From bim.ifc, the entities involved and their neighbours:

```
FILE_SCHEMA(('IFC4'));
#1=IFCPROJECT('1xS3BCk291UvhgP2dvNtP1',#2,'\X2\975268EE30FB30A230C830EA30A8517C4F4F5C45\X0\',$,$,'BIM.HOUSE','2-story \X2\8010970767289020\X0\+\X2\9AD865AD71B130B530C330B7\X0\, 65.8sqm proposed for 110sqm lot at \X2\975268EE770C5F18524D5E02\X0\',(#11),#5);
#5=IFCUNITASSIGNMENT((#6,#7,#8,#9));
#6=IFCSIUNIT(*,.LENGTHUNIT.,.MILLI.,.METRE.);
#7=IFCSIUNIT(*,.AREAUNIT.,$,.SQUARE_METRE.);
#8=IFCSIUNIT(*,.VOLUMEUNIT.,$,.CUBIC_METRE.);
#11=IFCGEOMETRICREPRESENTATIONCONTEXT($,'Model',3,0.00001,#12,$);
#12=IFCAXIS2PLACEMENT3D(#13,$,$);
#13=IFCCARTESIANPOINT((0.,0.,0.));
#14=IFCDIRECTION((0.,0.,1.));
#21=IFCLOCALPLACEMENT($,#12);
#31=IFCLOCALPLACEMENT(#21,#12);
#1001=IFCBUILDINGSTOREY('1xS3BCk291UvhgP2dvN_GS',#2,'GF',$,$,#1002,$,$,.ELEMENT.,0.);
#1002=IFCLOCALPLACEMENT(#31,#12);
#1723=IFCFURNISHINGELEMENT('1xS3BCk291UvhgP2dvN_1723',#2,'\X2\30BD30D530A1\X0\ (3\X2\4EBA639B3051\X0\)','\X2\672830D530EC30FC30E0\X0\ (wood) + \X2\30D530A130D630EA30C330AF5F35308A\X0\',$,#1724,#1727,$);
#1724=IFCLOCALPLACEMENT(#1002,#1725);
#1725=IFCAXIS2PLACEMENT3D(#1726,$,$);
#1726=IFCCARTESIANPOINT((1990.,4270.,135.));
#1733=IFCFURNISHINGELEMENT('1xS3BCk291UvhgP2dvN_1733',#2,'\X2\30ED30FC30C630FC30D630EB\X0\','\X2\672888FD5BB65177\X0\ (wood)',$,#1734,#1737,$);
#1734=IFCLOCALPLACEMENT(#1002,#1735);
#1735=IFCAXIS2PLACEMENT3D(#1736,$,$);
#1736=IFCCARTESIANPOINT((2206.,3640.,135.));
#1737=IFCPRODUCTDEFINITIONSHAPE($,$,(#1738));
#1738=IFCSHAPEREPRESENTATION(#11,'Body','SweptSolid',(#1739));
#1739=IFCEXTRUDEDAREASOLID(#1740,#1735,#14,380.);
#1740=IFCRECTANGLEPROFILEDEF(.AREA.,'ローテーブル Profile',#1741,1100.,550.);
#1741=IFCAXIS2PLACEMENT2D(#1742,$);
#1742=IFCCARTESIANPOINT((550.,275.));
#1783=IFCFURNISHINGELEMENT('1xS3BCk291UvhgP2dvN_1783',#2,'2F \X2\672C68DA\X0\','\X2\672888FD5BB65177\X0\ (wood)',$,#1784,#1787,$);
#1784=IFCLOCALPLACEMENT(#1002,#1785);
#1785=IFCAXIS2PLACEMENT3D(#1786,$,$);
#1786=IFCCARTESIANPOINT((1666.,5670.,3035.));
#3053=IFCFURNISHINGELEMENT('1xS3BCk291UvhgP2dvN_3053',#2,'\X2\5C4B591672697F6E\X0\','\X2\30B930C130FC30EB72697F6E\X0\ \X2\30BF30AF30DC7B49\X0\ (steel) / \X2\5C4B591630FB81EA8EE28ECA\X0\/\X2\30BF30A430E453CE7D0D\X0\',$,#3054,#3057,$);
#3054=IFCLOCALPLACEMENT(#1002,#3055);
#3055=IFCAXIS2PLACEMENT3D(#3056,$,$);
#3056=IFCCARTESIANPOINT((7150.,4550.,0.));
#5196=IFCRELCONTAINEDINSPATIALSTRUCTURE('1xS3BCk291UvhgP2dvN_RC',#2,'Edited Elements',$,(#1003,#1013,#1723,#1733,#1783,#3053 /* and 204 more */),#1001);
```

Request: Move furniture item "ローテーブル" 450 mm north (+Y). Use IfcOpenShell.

```python
import ifcopenshell
import ifcopenshell.api.geometry
import ifcopenshell.util.placement
import ifcopenshell.util.unit

model = ifcopenshell.open("bim.ifc")
unit_scale = ifcopenshell.util.unit.calculate_unit_scale(model)

item = model.by_id(1733)
matrix = ifcopenshell.util.placement.get_local_placement(item.ObjectPlacement)
matrix[1, 3] += 0.45 / unit_scale
ifcopenshell.api.geometry.edit_object_placement(model, product=item, matrix=matrix, is_si=False)

print(ifcopenshell.util.placement.get_local_placement(item.ObjectPlacement).round(3) + 0.0)

model.write("bim_rev.ifc")
```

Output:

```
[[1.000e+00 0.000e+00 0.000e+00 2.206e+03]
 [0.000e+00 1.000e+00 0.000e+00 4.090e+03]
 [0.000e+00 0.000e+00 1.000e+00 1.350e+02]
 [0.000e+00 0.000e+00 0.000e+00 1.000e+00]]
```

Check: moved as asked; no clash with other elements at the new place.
